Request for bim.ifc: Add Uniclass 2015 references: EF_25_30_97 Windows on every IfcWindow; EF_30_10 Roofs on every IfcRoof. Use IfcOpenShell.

First a look at what the model holds.

```python
import ifcopenshell

model = ifcopenshell.open("bim.ifc")
print(model.schema)
print("classifications:", [c.Name for c in model.by_type("IfcClassification")])
for ifc_class in ("IfcDoor", "IfcRoof", "IfcStair", "IfcWall", "IfcWindow"):
    print(ifc_class, len(model.by_type(ifc_class)))
```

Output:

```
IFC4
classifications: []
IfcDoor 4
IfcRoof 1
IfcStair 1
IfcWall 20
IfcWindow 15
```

```python
import ifcopenshell
import ifcopenshell.api.classification

model = ifcopenshell.open("bim.ifc")

system = ifcopenshell.api.classification.add_classification(model, classification="Uniclass 2015")

codes = {
    "IfcWindow": ("EF_25_30_97", "Windows"),
    "IfcRoof": ("EF_30_10", "Roofs"),
}
for ifc_class, (code, name) in codes.items():
    products = model.by_type(ifc_class)
    ifcopenshell.api.classification.add_reference(
        model, products=products, classification=system, identification=code, name=name
    )
    print(code, len(products))

model.write("bim_edited.ifc")
```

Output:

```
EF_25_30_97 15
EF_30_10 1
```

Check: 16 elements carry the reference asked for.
